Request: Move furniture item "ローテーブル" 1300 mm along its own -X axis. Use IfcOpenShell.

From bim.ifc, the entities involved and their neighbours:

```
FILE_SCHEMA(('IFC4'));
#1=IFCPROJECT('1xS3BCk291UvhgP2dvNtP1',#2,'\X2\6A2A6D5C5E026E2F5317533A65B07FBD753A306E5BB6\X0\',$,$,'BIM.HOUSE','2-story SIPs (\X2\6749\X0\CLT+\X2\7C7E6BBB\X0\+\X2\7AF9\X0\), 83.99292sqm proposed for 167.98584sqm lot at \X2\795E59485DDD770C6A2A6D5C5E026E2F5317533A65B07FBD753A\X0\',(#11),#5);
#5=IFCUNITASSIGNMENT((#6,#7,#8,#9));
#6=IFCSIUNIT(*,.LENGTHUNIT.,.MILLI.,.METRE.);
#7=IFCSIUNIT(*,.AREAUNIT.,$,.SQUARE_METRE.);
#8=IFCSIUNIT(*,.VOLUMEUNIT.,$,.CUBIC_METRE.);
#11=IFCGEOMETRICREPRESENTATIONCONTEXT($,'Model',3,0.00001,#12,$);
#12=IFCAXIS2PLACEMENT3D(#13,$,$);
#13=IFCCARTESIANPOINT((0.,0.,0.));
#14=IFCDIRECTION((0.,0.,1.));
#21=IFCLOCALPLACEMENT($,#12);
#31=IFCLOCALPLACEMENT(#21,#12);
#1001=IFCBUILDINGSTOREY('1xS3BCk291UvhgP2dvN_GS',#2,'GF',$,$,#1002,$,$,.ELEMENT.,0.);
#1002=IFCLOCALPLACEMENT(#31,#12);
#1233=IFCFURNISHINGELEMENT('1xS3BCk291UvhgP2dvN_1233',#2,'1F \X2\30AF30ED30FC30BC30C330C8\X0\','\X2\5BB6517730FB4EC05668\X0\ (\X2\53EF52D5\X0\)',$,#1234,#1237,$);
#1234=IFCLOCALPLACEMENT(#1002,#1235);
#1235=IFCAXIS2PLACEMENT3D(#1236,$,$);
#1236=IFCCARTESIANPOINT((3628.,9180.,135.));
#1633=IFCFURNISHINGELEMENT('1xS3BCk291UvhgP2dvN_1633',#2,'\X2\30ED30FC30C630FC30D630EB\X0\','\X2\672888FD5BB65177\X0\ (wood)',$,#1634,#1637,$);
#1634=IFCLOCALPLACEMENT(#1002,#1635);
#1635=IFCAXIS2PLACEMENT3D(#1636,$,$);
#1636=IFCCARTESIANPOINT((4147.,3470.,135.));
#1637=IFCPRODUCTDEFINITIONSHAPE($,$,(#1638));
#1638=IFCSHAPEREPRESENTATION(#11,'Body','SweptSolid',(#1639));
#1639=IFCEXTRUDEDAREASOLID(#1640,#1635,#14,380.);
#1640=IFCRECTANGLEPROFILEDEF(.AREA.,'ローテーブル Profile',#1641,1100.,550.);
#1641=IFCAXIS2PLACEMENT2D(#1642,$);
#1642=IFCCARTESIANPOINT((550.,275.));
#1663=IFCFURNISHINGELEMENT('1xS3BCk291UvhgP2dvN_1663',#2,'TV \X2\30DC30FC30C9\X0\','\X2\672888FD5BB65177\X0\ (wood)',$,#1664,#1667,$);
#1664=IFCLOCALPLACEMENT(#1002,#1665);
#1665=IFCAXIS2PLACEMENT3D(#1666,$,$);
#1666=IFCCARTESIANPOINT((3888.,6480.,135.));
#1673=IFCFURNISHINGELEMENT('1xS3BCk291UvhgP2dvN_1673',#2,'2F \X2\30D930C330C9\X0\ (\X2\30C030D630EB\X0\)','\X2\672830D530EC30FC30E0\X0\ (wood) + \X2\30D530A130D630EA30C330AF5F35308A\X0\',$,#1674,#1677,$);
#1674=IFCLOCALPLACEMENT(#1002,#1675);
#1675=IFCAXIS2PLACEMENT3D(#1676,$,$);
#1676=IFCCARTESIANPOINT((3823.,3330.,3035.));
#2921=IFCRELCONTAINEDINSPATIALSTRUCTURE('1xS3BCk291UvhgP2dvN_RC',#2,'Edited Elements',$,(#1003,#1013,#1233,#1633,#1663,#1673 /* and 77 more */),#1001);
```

```python
import ifcopenshell
import ifcopenshell.api.geometry
import ifcopenshell.util.placement
import ifcopenshell.util.unit

model = ifcopenshell.open("bim.ifc")
unit_scale = ifcopenshell.util.unit.calculate_unit_scale(model)

item = model.by_guid("1xS3BCk291UvhgP2dvN_1633")
matrix = ifcopenshell.util.placement.get_local_placement(item.ObjectPlacement)
matrix[:3, 3] -= matrix[:3, 0] * 1.3 / unit_scale
ifcopenshell.api.geometry.edit_object_placement(model, product=item, matrix=matrix, is_si=False)

print(ifcopenshell.util.placement.get_local_placement(item.ObjectPlacement).round(3) + 0.0)

model.write("bim_v2.ifc")
```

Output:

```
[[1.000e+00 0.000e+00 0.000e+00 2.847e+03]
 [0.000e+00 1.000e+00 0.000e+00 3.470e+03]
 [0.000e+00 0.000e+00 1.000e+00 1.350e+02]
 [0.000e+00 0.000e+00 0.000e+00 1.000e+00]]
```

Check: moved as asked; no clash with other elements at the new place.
